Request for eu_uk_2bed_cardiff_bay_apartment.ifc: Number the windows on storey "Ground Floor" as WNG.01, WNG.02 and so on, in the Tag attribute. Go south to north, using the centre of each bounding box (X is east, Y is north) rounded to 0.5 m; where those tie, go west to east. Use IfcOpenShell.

First a look at what the model holds.

```python
import ifcopenshell
import ifcopenshell.util.element
import ifcopenshell.util.placement

model = ifcopenshell.open("eu_uk_2bed_cardiff_bay_apartment.ifc")
print(model.schema)
storey = next(s for s in model.by_type("IfcBuildingStorey") if s.Name == "Ground Floor")
windows = [e for e in ifcopenshell.util.element.get_decomposition(storey) if e.is_a("IfcWindow")]
for e in sorted(windows, key=lambda e: e.id()):
    origin = ifcopenshell.util.placement.get_local_placement(e.ObjectPlacement)[:3, 3]
    print(e.id(), e.Tag, e.Name, origin.round(2) + 0.0, sep=" | ")
```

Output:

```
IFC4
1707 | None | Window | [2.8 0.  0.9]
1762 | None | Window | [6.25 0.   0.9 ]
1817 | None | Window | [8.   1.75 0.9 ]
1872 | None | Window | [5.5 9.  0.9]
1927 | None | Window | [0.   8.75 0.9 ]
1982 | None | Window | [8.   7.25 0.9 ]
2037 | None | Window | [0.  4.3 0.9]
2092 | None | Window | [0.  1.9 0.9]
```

```python
import ifcopenshell
import ifcopenshell.geom
import ifcopenshell.util.element
import ifcopenshell.util.shape

model = ifcopenshell.open("eu_uk_2bed_cardiff_bay_apartment.ifc")
settings = ifcopenshell.geom.settings()
settings.set("use-world-coords", True)


def centre(element):
    shape = ifcopenshell.geom.create_shape(settings, element)
    return ifcopenshell.util.shape.get_bbox_centroid(shape.geometry)


storey = next(s for s in model.by_type("IfcBuildingStorey") if s.Name == "Ground Floor")
windows = [e for e in ifcopenshell.util.element.get_decomposition(storey) if e.is_a("IfcWindow")]

# Insertion points can sit at a corner or the storey origin, so sort by the geometry (in metres).
centres = {e: centre(e) for e in windows}
windows.sort(key=lambda e: (round(centres[e][1] / 0.5), centres[e][0]))

for i, e in enumerate(windows, start=1):
    number = f"WNG.{i:02d}"
    e.Tag = number
    print(e.id(), number)

model.write("eu_uk_2bed_cardiff_bay_apartment_v2.ifc")
```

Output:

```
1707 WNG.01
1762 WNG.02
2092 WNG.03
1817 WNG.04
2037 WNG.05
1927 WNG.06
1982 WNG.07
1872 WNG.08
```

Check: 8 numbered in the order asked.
